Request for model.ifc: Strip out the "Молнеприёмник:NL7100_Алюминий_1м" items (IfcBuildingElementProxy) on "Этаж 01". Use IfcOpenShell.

First a look at what the model holds.

```python
import ifcopenshell
import ifcopenshell.util.element

model = ifcopenshell.open("model.ifc")
print(model.schema)
storey = next(s for s in model.by_type("IfcBuildingStorey") if s.Name == "Этаж 01")
proxies = [e for e in ifcopenshell.util.element.get_decomposition(storey) if e.is_a("IfcBuildingElementProxy")]
seen = {}
for e in proxies:
    element_type = ifcopenshell.util.element.get_type(e)
    name = element_type.Name if element_type not in (None, e) else None
    seen[name] = seen.get(name, 0) + 1
for name, count in sorted(seen.items(), key=str):
    print(count, "x", name)
```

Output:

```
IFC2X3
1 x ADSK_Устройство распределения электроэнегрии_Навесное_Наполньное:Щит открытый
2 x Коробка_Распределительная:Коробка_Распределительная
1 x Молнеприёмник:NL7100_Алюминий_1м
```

```python
import ifcopenshell
import ifcopenshell.api.root
import ifcopenshell.util.element

model = ifcopenshell.open("model.ifc")

storey = next(s for s in model.by_type("IfcBuildingStorey") if s.Name == "Этаж 01")
proxies = [e for e in ifcopenshell.util.element.get_decomposition(storey) if e.is_a("IfcBuildingElementProxy")]
targets = [e for e in proxies if (t := ifcopenshell.util.element.get_type(e)) not in (None, e) and t.Name == "Молнеприёмник:NL7100_Алюминий_1м"]

for e in targets:
    ifcopenshell.api.root.remove_product(model, product=e)
print(len(targets), "removed")

model.write("model-out.ifc")
```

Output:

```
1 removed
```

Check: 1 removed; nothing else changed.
